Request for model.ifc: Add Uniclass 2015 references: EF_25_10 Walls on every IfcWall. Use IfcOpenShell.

First a look at what the model holds.

```python
import ifcopenshell

model = ifcopenshell.open("model.ifc")
print(model.schema)
print("classifications:", [c.Name for c in model.by_type("IfcClassification")])
for ifc_class in ("IfcDoor", "IfcRoof", "IfcStair", "IfcWall", "IfcWindow"):
    print(ifc_class, len(model.by_type(ifc_class)))
```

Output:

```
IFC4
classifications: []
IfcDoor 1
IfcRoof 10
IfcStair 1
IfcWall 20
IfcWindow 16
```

```python
import ifcopenshell
import ifcopenshell.api.classification

model = ifcopenshell.open("model.ifc")

system = ifcopenshell.api.classification.add_classification(model, classification="Uniclass 2015")

codes = {
    "IfcWall": ("EF_25_10", "Walls"),
}
for ifc_class, (code, name) in codes.items():
    products = model.by_type(ifc_class)
    ifcopenshell.api.classification.add_reference(
        model, products=products, classification=system, identification=code, name=name
    )
    print(code, len(products))

model.write("model_edited.ifc")
```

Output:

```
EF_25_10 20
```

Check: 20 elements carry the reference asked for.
